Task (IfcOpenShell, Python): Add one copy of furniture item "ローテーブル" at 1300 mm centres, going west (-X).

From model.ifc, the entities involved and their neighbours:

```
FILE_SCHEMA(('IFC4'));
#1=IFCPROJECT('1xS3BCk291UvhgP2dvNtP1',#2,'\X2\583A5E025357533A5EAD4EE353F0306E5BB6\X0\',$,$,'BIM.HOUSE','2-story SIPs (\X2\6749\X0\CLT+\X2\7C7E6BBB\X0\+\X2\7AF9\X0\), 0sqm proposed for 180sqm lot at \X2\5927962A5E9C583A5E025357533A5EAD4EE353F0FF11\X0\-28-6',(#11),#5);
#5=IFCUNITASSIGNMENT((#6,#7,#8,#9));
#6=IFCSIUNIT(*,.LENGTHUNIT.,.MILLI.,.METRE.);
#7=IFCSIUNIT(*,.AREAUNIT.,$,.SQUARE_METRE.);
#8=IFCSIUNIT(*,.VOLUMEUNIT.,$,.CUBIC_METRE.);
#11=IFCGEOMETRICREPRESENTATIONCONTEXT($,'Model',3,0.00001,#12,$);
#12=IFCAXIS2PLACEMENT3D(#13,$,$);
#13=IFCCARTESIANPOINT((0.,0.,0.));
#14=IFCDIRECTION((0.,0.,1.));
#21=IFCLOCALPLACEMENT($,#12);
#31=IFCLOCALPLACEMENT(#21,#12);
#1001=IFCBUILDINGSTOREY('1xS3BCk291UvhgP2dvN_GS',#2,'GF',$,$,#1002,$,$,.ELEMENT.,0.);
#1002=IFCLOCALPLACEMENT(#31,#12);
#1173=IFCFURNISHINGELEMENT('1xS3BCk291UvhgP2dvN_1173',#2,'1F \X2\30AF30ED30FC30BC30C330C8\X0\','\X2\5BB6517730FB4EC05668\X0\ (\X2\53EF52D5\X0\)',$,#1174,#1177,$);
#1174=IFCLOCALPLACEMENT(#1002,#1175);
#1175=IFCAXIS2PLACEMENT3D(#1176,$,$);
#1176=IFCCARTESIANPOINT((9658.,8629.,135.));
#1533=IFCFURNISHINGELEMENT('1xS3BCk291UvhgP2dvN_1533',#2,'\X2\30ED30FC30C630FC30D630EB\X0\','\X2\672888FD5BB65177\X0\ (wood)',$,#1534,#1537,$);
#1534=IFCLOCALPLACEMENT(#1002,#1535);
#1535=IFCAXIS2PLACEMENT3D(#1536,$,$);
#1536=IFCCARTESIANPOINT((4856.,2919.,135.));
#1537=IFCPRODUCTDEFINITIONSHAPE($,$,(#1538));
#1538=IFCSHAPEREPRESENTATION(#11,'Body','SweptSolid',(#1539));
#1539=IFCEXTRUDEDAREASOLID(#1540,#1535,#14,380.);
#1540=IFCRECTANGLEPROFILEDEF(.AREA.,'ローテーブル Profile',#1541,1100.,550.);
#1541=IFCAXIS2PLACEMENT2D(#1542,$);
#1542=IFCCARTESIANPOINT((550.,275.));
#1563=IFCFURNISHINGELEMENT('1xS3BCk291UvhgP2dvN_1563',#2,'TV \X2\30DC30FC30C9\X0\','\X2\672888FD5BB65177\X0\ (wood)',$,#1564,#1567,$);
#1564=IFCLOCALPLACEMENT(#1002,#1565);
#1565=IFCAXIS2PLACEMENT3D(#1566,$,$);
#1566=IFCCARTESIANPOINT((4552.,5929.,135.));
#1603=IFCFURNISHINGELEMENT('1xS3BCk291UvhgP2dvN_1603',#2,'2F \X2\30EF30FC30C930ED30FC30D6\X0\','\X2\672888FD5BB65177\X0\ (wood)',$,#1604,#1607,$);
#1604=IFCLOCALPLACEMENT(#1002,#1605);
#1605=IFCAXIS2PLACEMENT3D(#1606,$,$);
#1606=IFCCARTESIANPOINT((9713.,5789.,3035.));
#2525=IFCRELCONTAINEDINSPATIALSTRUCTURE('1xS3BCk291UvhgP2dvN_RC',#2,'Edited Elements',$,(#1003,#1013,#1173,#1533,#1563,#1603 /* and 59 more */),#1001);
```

```python
import numpy as np
import ifcopenshell
import ifcopenshell.api.geometry
import ifcopenshell.api.root
import ifcopenshell.util.element
import ifcopenshell.util.placement
import ifcopenshell.util.unit

model = ifcopenshell.open("model.ifc")
unit_scale = ifcopenshell.util.unit.calculate_unit_scale(model)


def reuse_history(source, copy):
    """copy_class also copies each property set's owner history, people and application; keep the originals."""
    for rel in copy.IsDefinedBy:
        if rel.is_a("IfcRelDefinesByProperties") and (history := rel.RelatingPropertyDefinition.OwnerHistory):
            rel.RelatingPropertyDefinition.OwnerHistory = source.OwnerHistory
            ifcopenshell.util.element.remove_deep2(model, history)


source = model.by_guid("1xS3BCk291UvhgP2dvN_1533")
base = ifcopenshell.util.placement.get_local_placement(source.ObjectPlacement)
step = np.array([-1.0, 0.0, 0.0]) * 1.3 / unit_scale

for i in range(1, 2):
    copy = ifcopenshell.api.root.copy_class(model, product=source)
    copy.Representation = ifcopenshell.util.element.copy_deep(
        model, source.Representation, exclude=["IfcGeometricRepresentationContext", "IfcRepresentationMap"]
    )
    reuse_history(source, copy)
    matrix = base.copy()
    matrix[:3, 3] += i * step
    print("added at", matrix[:3, 3].round(3) + 0.0)
    ifcopenshell.api.geometry.edit_object_placement(model, product=copy, matrix=matrix, is_si=False)

model.write("model_edited.ifc")
```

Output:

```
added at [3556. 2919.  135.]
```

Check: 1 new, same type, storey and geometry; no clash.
